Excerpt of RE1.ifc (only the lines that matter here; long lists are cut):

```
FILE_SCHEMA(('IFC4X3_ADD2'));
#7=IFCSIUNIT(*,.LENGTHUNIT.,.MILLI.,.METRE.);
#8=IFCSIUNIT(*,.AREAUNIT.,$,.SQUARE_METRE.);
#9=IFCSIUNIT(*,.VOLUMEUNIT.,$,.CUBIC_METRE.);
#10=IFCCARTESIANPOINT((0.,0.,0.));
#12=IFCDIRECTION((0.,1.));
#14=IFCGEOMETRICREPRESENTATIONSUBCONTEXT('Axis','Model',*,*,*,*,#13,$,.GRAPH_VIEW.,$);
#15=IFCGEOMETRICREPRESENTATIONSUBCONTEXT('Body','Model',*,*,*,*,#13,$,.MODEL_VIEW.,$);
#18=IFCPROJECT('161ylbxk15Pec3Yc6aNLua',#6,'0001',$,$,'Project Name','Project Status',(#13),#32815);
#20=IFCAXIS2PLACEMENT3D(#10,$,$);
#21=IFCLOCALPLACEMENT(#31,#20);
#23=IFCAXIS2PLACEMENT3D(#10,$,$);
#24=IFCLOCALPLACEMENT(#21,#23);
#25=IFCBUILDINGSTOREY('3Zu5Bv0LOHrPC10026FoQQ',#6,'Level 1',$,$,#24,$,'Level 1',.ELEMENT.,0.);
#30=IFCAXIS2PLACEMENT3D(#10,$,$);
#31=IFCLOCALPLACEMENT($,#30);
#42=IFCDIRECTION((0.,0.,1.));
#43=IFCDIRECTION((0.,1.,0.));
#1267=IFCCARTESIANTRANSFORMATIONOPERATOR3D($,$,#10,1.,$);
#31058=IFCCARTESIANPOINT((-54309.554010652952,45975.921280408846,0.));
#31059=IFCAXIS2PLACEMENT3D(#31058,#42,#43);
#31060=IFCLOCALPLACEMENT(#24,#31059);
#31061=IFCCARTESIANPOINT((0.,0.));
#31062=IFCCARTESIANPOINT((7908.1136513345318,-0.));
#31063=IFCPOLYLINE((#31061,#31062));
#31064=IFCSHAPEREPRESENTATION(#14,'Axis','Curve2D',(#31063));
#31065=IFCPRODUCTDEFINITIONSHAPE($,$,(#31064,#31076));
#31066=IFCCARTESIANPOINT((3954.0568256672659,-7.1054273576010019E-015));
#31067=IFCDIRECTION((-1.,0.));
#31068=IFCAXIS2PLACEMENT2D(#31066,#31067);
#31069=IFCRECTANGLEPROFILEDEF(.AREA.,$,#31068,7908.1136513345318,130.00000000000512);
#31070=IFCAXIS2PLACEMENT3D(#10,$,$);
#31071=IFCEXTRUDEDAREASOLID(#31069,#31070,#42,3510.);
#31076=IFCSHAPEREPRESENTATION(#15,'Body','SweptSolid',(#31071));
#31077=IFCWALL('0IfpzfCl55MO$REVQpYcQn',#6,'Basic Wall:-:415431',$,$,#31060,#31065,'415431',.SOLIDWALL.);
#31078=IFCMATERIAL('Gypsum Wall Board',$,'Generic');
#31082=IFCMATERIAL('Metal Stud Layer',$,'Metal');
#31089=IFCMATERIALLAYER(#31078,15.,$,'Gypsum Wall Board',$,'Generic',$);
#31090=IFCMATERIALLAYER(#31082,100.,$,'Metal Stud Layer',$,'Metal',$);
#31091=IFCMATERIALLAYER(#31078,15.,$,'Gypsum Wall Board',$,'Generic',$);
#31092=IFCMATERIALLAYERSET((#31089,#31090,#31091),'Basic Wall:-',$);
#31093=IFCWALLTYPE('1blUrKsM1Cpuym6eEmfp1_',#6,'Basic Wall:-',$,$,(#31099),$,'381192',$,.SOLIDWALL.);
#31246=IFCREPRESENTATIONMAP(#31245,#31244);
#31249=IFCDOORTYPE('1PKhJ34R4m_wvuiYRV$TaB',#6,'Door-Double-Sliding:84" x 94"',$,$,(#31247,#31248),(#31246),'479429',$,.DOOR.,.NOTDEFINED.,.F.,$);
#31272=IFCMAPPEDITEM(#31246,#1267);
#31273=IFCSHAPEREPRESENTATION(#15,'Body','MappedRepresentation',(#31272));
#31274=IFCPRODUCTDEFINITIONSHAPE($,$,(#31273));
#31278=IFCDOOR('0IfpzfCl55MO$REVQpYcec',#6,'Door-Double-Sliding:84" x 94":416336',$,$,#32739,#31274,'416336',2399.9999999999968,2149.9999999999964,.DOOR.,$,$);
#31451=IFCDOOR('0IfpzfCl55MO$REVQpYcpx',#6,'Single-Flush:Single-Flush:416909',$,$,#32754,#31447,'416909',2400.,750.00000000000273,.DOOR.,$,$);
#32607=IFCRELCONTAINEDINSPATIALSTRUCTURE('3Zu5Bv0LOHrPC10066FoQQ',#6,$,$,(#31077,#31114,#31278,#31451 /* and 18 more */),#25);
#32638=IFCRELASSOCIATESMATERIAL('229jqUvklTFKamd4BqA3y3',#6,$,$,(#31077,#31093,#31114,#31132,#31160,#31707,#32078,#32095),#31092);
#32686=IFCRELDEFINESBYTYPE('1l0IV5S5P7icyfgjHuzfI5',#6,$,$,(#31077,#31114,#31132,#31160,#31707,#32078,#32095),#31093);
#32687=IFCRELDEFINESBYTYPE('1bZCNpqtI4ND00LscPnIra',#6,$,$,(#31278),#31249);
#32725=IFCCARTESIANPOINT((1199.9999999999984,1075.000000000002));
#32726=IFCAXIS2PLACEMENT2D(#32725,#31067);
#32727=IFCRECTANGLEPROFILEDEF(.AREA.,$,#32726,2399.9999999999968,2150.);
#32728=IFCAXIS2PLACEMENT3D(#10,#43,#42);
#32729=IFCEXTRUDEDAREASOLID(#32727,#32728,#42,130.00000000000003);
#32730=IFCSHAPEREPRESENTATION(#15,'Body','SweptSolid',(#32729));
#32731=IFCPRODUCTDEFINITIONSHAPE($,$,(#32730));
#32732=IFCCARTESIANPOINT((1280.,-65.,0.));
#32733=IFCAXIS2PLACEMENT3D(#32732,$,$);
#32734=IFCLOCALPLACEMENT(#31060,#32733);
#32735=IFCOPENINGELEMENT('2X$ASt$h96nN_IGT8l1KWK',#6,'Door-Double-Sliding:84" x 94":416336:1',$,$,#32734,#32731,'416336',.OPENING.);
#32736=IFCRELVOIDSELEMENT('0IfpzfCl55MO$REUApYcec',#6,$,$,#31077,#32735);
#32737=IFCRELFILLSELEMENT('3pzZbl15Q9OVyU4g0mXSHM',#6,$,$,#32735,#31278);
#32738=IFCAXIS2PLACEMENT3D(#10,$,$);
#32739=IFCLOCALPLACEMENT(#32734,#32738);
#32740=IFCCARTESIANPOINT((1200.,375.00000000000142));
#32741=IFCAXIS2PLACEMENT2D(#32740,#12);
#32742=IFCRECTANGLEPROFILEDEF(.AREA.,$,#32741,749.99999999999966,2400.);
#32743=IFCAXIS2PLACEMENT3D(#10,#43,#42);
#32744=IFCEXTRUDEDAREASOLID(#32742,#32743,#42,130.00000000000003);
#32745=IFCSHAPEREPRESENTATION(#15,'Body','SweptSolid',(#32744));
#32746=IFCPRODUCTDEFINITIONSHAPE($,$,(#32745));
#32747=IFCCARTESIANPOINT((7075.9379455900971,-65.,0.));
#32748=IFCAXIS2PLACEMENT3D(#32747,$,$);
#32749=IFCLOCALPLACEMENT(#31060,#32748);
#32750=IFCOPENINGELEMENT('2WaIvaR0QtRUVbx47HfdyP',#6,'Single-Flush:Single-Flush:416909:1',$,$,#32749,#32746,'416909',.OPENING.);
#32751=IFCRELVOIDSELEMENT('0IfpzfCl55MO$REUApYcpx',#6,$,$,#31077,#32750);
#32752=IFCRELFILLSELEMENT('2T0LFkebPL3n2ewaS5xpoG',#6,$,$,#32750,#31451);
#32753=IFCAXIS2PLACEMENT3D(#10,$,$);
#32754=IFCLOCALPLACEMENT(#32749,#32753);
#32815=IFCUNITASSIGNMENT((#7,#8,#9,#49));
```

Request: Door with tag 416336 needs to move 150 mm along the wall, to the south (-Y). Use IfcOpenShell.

```python
import ifcopenshell
import ifcopenshell.api.geometry
import ifcopenshell.util.placement
import ifcopenshell.util.unit

model = ifcopenshell.open("RE1.ifc")
unit_scale = ifcopenshell.util.unit.calculate_unit_scale(model)

door = model.by_guid("0IfpzfCl55MO$REVQpYcec")
opening = door.FillsVoids[0].RelatingOpeningElement
wall = opening.VoidsElements[0].RelatingBuildingElement

wall_matrix = ifcopenshell.util.placement.get_local_placement(wall.ObjectPlacement)
shift = wall_matrix[:3, 0] * -0.15 / unit_scale
before = ifcopenshell.util.placement.get_local_placement(door.ObjectPlacement)[:3, 3].copy()

# The door is placed relative to its opening, so it follows when the opening moves.
matrix = ifcopenshell.util.placement.get_local_placement(opening.ObjectPlacement)
matrix[:3, 3] += shift
ifcopenshell.api.geometry.edit_object_placement(
    model, product=opening, matrix=matrix, is_si=False, should_transform_children=True
)

after = ifcopenshell.util.placement.get_local_placement(door.ObjectPlacement)[:3, 3]
print("door moved by", (after - before).round(3) + 0.0)

model.write("RE1_v2.ifc")
```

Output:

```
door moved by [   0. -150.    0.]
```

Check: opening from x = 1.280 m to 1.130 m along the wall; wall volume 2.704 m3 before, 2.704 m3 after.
